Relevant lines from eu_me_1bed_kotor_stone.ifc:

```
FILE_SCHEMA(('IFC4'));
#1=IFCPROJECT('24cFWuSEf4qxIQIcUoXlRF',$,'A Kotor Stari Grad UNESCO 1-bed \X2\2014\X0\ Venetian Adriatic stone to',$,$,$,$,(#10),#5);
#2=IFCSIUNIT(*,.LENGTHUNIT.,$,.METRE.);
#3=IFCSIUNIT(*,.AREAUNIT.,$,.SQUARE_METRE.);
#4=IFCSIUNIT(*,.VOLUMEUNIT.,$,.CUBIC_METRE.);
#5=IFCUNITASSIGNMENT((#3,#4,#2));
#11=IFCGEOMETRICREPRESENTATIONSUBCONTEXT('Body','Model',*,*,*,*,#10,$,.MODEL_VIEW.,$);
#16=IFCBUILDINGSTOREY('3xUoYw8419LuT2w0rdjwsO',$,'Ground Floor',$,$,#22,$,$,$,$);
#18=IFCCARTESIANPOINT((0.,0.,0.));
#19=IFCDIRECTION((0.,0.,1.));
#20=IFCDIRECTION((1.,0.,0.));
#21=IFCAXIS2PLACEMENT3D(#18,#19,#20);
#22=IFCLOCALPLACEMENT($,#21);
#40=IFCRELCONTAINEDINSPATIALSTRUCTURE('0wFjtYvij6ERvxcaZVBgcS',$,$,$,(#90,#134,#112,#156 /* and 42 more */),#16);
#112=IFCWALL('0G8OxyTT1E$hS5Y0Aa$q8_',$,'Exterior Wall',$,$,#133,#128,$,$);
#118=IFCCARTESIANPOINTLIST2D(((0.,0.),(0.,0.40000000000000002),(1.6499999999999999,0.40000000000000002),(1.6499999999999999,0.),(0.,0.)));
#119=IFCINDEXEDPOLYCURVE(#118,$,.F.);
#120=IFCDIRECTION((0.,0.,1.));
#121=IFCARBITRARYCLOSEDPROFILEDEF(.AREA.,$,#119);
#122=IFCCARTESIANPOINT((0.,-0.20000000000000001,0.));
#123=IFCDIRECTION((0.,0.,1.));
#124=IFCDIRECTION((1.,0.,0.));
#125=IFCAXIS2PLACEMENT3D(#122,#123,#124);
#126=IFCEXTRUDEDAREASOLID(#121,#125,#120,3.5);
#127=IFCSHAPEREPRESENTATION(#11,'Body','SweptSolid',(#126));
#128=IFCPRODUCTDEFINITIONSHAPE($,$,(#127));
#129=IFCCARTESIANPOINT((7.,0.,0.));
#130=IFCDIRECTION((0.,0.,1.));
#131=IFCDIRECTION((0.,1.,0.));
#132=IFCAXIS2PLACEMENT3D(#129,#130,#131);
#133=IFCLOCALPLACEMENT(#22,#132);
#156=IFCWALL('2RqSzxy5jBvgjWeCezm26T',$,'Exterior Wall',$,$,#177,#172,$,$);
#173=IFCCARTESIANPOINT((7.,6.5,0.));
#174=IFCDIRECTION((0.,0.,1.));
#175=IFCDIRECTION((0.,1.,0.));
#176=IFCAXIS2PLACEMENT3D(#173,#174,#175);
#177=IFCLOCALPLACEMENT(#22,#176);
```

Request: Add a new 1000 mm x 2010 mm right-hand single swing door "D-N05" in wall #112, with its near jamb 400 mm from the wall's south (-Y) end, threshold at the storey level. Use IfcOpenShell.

```python
import numpy as np
import ifcopenshell
import ifcopenshell.api.feature
import ifcopenshell.api.geometry
import ifcopenshell.api.root
import ifcopenshell.api.spatial
import ifcopenshell.geom
import ifcopenshell.util.element
import ifcopenshell.util.placement
import ifcopenshell.util.representation
import ifcopenshell.util.shape
import ifcopenshell.util.unit

model = ifcopenshell.open("eu_me_1bed_kotor_stone.ifc")
unit_scale = ifcopenshell.util.unit.calculate_unit_scale(model)
settings = ifcopenshell.geom.settings()


def volume(element):
    """Net volume in cubic metres, openings subtracted."""
    shape = ifcopenshell.geom.create_shape(settings, element)
    return ifcopenshell.util.shape.get_volume(shape.geometry)


wall = model.by_id(112)
storey = ifcopenshell.util.element.get_container(wall, ifc_class="IfcBuildingStorey")
context = ifcopenshell.util.representation.get_context(model, "Model", "Body", "MODEL_VIEW")
before = volume(wall)

width, height, from_end, sill = 1, 2.01, 0.4, 0.0  # metres

# The wall runs along its own X axis, and the end named is its -X end.
wall_shape = ifcopenshell.geom.create_shape(settings, wall)
x, y, z = ifcopenshell.util.shape.get_vertices(wall_shape.geometry).T
start = x.min() + from_end
face, thickness = float(y.min()), float(y.max() - y.min())
wall_matrix = ifcopenshell.util.placement.get_local_placement(wall.ObjectPlacement)
level = ifcopenshell.util.placement.get_local_placement(storey.ObjectPlacement)[2, 3]


def in_wall(x, y):
    """Placement at x, y metres in the wall's axes, at sill height."""
    matrix = wall_matrix.copy()
    matrix[:, 3] = wall_matrix @ np.array([x / unit_scale, y / unit_scale, 0.0, 1.0])
    matrix[2, 3] = level + sill / unit_scale
    return matrix


# Opening: a box that overshoots both wall faces by 50 mm.
opening = ifcopenshell.api.root.create_entity(model, ifc_class="IfcOpeningElement", predefined_type="OPENING")
box = ifcopenshell.api.geometry.add_wall_representation(
    model, context=context, length=width, height=height, thickness=thickness + 0.1
)
ifcopenshell.api.geometry.assign_representation(model, product=opening, representation=box)
ifcopenshell.api.geometry.edit_object_placement(model, product=opening, matrix=in_wall(start, face - 0.05), is_si=False)
ifcopenshell.api.feature.add_feature(model, feature=opening, element=wall)

door = ifcopenshell.api.root.create_entity(model, ifc_class="IfcDoor", name="D-N05", predefined_type="DOOR")
door.OverallWidth, door.OverallHeight = width / unit_scale, height / unit_scale
door.OperationType = "SINGLE_SWING_RIGHT"
body = ifcopenshell.api.geometry.add_door_representation(
    model,
    context=context,
    overall_width=door.OverallWidth,
    overall_height=door.OverallHeight,
    operation_type="SINGLE_SWING_RIGHT",
    lining_properties={"LiningDepth": thickness / unit_scale, "ThresholdDepth": thickness / unit_scale},
)
ifcopenshell.api.geometry.assign_representation(model, product=door, representation=body)
ifcopenshell.api.spatial.assign_container(model, products=[door], relating_structure=storey)
ifcopenshell.api.feature.add_filling(model, opening=opening, element=door)

# The lining spans the wall, so the door starts at the wall face.
ifcopenshell.api.geometry.edit_object_placement(model, product=door, matrix=in_wall(start, face), is_si=False)

after = volume(wall)

print(f"wall volume {before:.3f} -> {after:.3f} m3")

model.write("eu_me_1bed_kotor_stone_edited.ifc")
```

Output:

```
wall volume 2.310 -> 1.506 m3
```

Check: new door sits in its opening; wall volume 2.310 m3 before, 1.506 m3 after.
